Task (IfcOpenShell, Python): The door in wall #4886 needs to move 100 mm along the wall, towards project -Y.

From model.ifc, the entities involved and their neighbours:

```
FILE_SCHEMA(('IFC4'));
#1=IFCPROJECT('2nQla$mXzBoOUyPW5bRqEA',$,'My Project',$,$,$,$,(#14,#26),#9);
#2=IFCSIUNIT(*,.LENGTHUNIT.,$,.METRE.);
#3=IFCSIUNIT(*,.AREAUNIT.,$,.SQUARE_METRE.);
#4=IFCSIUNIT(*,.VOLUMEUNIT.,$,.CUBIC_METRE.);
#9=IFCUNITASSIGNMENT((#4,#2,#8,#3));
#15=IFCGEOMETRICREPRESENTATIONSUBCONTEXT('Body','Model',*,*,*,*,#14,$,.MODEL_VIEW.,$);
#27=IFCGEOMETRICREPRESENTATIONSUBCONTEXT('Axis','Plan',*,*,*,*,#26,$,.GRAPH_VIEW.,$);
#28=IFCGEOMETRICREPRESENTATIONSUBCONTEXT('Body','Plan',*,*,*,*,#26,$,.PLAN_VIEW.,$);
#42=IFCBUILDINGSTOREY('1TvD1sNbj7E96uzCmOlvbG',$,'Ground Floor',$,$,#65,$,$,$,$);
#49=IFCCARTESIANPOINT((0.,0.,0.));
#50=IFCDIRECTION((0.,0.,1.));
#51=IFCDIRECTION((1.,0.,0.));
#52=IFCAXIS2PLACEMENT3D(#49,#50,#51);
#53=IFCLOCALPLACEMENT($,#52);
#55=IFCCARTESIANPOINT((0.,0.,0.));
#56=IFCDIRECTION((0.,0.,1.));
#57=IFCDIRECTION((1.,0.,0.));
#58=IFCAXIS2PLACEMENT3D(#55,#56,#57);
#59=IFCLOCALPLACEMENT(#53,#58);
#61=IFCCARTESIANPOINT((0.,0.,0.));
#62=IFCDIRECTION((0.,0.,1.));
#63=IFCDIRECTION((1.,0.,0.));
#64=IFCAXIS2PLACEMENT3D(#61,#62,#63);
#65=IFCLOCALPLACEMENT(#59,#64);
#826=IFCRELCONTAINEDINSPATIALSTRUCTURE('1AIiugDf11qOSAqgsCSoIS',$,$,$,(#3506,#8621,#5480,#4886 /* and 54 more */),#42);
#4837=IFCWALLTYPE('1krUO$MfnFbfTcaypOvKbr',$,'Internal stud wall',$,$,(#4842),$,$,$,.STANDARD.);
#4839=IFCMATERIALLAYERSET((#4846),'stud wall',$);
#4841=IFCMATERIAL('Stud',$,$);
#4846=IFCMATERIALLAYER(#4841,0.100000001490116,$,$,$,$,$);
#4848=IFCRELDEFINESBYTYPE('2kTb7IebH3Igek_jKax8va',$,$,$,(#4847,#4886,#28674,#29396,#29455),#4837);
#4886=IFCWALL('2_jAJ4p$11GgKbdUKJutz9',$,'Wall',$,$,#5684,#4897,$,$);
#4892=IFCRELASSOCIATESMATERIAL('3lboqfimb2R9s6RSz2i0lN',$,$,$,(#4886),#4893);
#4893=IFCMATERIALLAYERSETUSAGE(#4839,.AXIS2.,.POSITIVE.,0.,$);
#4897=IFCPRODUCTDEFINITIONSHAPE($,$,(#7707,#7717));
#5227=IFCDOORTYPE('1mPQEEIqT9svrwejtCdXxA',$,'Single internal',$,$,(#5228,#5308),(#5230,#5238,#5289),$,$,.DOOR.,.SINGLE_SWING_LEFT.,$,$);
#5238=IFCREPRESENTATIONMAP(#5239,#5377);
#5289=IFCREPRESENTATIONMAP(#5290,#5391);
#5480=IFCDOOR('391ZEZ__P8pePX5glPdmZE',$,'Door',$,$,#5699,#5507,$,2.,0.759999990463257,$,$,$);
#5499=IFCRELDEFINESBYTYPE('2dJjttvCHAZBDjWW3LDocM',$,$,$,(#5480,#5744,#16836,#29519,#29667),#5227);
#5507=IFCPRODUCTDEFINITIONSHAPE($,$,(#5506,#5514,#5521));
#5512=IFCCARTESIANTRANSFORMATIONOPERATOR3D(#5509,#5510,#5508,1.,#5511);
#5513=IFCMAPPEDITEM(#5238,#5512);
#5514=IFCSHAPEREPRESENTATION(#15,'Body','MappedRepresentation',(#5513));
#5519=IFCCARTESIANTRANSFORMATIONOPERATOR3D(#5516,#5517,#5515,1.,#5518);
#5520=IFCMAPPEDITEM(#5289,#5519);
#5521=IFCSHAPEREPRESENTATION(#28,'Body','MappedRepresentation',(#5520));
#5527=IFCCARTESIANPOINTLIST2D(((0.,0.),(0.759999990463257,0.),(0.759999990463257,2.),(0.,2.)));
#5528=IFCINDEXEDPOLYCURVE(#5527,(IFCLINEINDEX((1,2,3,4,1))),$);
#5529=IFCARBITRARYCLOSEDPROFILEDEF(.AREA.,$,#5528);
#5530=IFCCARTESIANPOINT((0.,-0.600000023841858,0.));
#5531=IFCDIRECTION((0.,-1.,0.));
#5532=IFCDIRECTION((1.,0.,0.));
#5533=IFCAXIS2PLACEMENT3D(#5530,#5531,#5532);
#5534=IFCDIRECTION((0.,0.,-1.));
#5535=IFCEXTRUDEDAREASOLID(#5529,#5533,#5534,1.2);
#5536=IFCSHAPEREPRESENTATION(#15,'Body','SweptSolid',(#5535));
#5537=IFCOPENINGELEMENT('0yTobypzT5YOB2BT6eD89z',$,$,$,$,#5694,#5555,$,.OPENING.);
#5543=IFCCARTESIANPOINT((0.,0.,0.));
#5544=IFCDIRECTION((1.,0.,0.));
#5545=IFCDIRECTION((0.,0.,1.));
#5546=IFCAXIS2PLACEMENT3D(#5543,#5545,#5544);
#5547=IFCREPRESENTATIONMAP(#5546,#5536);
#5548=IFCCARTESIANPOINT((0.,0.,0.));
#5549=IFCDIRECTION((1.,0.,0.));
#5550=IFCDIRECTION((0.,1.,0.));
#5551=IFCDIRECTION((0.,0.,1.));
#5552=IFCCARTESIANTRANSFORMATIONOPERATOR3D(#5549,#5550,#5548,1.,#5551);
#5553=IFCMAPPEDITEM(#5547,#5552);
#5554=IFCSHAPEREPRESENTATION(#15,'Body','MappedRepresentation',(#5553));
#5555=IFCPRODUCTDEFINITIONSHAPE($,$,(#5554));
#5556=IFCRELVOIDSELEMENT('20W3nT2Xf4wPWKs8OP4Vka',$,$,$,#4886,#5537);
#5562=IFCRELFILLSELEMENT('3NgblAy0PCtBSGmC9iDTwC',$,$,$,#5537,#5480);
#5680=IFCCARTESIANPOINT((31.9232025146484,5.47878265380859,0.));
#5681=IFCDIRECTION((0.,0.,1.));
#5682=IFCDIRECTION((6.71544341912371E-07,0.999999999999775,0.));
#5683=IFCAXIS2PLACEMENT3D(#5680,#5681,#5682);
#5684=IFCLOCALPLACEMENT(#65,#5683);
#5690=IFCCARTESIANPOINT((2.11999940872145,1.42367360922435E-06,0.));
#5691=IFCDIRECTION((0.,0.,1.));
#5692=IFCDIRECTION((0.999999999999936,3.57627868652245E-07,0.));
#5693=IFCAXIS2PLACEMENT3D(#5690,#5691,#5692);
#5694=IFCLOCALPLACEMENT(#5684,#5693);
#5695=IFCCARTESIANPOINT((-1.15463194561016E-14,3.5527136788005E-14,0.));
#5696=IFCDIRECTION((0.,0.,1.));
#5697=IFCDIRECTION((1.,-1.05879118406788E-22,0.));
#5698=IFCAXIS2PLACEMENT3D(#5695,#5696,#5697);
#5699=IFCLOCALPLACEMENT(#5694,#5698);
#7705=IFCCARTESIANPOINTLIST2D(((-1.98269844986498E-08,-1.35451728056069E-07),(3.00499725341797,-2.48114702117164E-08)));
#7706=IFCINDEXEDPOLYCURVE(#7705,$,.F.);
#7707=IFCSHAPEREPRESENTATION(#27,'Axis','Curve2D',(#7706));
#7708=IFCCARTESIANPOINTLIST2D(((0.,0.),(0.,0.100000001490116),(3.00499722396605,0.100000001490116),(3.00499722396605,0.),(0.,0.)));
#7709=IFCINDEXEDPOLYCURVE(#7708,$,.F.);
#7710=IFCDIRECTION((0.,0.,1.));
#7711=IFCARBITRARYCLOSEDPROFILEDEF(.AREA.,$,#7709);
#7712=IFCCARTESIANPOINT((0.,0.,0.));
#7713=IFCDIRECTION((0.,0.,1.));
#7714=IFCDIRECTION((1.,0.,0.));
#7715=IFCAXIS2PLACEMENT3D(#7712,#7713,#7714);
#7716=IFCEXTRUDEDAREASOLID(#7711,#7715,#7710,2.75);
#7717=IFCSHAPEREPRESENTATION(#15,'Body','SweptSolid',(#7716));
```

```python
import ifcopenshell
import ifcopenshell.api.geometry
import ifcopenshell.util.placement

model = ifcopenshell.open("model.ifc")

door = model.by_guid("391ZEZ__P8pePX5glPdmZE")
opening = door.FillsVoids[0].RelatingOpeningElement
wall = opening.VoidsElements[0].RelatingBuildingElement

wall_matrix = ifcopenshell.util.placement.get_local_placement(wall.ObjectPlacement)
shift = wall_matrix[:3, 0] * -0.1
before = ifcopenshell.util.placement.get_local_placement(door.ObjectPlacement)[:3, 3].copy()

# The door is placed relative to its opening, so it follows when the opening moves.
matrix = ifcopenshell.util.placement.get_local_placement(opening.ObjectPlacement)
matrix[:3, 3] += shift
ifcopenshell.api.geometry.edit_object_placement(
    model, product=opening, matrix=matrix, is_si=False, should_transform_children=True
)

after = ifcopenshell.util.placement.get_local_placement(door.ObjectPlacement)[:3, 3]
print("door moved by", (after - before).round(3) + 0.0)

model.write("model_updated.ifc")
```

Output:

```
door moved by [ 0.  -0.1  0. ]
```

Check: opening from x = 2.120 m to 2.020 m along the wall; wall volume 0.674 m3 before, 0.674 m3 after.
